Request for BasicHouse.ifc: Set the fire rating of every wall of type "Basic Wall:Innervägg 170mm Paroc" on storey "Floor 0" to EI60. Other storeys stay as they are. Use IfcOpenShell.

First a look at what the model holds.

```python
import ifcopenshell
import ifcopenshell.util.element

model = ifcopenshell.open("BasicHouse.ifc")
print(model.schema)
storey = next(s for s in model.by_type("IfcBuildingStorey") if s.Name == "Floor 0")
walls = [e for e in ifcopenshell.util.element.get_decomposition(storey) if e.is_a("IfcWall")]
seen = {}
for e in walls:
    element_type = ifcopenshell.util.element.get_type(e)
    key = (element_type.Name if element_type != e and element_type else None, ifcopenshell.util.element.get_pset(e, "Pset_WallCommon", "FireRating"))
    seen[key] = seen.get(key, 0) + 1
for (name, value), count in sorted(seen.items(), key=str):
    print(count, "x", name, "|", value)
```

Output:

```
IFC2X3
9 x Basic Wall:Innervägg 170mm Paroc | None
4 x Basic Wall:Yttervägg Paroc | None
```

```python
import ifcopenshell
import ifcopenshell.api.pset
import ifcopenshell.util.element

model = ifcopenshell.open("BasicHouse.ifc")

storey = next(s for s in model.by_type("IfcBuildingStorey") if s.Name == "Floor 0")
walls = [e for e in ifcopenshell.util.element.get_decomposition(storey) if e.is_a("IfcWall")]

count = 0
for e in walls:
    element_type = ifcopenshell.util.element.get_type(e)
    if element_type in (None, e) or element_type.Name != "Basic Wall:Innervägg 170mm Paroc":
        continue
    # add_pset returns the element's existing set when there is one.
    pset = ifcopenshell.api.pset.add_pset(model, product=e, name="Pset_WallCommon")
    ifcopenshell.api.pset.edit_pset(model, pset=pset, properties={"FireRating": "EI60"})
    count += 1

print(count, "walls updated")

model.write("BasicHouse-out.ifc")
```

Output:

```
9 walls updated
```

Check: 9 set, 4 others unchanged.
